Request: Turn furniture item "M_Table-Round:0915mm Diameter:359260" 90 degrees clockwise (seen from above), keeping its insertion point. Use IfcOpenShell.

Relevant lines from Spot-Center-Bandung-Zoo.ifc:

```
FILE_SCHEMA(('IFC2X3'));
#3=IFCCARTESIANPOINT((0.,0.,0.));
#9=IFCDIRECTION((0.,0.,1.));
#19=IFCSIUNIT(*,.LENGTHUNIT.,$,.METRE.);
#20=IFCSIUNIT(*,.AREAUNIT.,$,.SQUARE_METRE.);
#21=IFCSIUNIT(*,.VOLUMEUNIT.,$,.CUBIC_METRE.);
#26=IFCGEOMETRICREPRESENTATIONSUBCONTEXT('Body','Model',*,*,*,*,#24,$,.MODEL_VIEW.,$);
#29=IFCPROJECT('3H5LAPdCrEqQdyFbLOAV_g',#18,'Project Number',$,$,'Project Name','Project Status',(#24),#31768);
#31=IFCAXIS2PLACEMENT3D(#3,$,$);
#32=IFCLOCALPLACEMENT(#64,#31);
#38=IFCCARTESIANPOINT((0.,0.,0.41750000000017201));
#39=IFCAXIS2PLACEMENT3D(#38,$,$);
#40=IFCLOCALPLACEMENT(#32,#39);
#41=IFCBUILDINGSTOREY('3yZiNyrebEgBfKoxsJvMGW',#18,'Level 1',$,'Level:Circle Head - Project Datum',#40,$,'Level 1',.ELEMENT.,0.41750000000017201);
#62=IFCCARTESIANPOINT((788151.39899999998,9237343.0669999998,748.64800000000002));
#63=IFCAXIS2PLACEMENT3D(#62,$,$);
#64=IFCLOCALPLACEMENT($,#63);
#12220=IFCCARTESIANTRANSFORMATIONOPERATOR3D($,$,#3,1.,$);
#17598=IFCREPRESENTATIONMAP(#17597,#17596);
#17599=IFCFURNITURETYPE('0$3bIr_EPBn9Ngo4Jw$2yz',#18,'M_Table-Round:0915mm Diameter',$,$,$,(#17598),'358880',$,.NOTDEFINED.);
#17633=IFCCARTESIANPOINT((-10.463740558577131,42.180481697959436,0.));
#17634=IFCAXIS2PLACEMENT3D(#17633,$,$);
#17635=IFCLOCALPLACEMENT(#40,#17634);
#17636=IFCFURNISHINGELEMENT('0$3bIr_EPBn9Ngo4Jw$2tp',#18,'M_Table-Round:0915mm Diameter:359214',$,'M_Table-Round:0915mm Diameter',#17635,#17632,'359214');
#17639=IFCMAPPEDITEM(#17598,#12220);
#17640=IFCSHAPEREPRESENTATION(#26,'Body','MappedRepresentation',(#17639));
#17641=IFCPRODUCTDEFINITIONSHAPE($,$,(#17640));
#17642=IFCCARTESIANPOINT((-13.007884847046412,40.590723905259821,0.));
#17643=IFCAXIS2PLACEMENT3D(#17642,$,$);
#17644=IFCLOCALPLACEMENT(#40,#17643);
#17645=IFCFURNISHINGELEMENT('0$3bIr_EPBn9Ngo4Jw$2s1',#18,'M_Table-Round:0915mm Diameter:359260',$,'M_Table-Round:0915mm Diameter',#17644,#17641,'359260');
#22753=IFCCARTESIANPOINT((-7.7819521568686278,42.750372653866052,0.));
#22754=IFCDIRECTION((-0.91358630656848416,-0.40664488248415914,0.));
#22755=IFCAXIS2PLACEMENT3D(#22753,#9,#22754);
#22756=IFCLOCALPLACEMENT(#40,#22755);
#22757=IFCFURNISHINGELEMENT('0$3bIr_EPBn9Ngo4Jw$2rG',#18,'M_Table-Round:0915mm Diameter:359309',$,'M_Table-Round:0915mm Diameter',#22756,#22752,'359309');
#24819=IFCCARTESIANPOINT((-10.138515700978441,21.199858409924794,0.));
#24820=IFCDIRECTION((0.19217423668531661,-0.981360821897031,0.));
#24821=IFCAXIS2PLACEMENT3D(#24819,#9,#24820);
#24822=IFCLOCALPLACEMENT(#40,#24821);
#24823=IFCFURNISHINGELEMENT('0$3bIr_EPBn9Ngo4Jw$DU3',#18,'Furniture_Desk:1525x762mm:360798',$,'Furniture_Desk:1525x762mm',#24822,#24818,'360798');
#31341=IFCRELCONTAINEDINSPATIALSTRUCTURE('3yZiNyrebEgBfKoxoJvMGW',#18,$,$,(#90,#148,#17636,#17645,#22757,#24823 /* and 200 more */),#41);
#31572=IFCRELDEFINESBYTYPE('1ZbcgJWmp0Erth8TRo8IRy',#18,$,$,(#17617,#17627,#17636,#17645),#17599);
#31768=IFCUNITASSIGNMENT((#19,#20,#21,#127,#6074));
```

```python
import ifcopenshell
import ifcopenshell.api.geometry
import ifcopenshell.util.placement

model = ifcopenshell.open("Spot-Center-Bandung-Zoo.ifc")

item = model.by_guid("0$3bIr_EPBn9Ngo4Jw$2s1")
matrix = ifcopenshell.util.placement.get_local_placement(item.ObjectPlacement)
matrix = matrix @ ifcopenshell.util.placement.rotation(-90, "Z")
ifcopenshell.api.geometry.edit_object_placement(model, product=item, matrix=matrix, is_si=False)

print(ifcopenshell.util.placement.get_local_placement(item.ObjectPlacement).round(3) + 0.0)

model.write("Spot-Center-Bandung-Zoo_updated.ifc")
```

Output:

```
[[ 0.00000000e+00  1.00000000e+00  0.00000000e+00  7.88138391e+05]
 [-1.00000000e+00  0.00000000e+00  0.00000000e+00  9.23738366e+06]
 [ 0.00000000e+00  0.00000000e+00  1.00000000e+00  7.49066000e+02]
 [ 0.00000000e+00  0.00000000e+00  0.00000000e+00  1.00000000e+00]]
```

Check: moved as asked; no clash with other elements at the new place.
